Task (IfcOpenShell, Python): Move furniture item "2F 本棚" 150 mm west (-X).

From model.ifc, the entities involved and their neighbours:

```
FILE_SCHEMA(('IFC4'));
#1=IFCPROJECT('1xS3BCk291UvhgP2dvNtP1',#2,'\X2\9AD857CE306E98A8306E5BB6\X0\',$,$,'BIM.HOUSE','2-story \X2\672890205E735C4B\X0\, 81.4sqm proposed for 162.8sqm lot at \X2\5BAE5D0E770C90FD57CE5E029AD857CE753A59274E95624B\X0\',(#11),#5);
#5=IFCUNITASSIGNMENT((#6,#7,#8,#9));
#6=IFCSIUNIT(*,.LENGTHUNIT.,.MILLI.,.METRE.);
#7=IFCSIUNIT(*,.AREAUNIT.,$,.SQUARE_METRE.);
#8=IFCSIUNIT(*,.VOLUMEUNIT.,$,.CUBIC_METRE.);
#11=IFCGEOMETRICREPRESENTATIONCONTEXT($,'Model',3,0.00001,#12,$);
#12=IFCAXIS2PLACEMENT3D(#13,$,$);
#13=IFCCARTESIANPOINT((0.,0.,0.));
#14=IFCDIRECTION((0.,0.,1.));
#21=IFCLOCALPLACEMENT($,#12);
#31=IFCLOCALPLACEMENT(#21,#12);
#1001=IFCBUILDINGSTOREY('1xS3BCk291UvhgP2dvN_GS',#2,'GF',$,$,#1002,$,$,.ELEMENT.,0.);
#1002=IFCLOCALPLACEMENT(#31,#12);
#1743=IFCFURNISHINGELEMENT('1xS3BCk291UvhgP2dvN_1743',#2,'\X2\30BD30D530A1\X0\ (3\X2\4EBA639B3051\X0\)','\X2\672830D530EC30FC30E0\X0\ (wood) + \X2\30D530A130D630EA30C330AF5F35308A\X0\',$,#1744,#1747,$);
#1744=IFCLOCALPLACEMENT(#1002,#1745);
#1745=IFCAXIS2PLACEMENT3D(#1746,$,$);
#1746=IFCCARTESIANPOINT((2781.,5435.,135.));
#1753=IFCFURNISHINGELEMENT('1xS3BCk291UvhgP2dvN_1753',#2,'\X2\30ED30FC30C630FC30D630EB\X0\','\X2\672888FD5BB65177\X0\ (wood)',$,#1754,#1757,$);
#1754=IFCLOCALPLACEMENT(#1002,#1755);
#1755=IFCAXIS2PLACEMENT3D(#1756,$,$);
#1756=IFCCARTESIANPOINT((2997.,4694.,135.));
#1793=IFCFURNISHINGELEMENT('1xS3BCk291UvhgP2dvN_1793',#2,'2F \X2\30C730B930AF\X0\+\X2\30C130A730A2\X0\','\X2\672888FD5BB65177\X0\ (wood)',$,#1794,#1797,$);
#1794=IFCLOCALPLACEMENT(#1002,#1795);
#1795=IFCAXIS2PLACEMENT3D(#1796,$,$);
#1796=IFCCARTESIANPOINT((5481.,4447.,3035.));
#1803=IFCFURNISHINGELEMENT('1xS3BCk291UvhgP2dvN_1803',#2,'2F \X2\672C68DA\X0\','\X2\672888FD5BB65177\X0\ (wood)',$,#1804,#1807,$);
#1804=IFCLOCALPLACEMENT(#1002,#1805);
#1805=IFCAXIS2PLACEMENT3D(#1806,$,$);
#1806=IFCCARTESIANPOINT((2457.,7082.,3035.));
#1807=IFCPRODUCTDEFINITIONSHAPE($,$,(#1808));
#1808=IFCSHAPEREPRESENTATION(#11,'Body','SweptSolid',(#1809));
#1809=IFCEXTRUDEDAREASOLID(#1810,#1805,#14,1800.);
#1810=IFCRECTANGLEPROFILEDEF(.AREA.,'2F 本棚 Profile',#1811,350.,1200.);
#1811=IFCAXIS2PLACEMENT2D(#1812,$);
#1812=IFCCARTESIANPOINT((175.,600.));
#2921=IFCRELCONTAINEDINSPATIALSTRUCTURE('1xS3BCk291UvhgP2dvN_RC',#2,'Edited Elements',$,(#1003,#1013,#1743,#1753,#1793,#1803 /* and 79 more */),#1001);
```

```python
import ifcopenshell
import ifcopenshell.api.geometry
import ifcopenshell.util.placement

model = ifcopenshell.open("model.ifc")

item = model.by_guid("1xS3BCk291UvhgP2dvN_1803")
matrix = ifcopenshell.util.placement.get_local_placement(item.ObjectPlacement)
matrix[0, 3] -= 150.0
ifcopenshell.api.geometry.edit_object_placement(model, product=item, matrix=matrix, is_si=False)

print(ifcopenshell.util.placement.get_local_placement(item.ObjectPlacement).round(3) + 0.0)

model.write("model_edited.ifc")
```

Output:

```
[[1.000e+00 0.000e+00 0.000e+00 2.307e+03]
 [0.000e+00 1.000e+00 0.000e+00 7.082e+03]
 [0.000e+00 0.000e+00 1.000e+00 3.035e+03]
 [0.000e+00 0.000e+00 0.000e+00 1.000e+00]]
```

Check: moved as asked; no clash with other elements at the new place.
